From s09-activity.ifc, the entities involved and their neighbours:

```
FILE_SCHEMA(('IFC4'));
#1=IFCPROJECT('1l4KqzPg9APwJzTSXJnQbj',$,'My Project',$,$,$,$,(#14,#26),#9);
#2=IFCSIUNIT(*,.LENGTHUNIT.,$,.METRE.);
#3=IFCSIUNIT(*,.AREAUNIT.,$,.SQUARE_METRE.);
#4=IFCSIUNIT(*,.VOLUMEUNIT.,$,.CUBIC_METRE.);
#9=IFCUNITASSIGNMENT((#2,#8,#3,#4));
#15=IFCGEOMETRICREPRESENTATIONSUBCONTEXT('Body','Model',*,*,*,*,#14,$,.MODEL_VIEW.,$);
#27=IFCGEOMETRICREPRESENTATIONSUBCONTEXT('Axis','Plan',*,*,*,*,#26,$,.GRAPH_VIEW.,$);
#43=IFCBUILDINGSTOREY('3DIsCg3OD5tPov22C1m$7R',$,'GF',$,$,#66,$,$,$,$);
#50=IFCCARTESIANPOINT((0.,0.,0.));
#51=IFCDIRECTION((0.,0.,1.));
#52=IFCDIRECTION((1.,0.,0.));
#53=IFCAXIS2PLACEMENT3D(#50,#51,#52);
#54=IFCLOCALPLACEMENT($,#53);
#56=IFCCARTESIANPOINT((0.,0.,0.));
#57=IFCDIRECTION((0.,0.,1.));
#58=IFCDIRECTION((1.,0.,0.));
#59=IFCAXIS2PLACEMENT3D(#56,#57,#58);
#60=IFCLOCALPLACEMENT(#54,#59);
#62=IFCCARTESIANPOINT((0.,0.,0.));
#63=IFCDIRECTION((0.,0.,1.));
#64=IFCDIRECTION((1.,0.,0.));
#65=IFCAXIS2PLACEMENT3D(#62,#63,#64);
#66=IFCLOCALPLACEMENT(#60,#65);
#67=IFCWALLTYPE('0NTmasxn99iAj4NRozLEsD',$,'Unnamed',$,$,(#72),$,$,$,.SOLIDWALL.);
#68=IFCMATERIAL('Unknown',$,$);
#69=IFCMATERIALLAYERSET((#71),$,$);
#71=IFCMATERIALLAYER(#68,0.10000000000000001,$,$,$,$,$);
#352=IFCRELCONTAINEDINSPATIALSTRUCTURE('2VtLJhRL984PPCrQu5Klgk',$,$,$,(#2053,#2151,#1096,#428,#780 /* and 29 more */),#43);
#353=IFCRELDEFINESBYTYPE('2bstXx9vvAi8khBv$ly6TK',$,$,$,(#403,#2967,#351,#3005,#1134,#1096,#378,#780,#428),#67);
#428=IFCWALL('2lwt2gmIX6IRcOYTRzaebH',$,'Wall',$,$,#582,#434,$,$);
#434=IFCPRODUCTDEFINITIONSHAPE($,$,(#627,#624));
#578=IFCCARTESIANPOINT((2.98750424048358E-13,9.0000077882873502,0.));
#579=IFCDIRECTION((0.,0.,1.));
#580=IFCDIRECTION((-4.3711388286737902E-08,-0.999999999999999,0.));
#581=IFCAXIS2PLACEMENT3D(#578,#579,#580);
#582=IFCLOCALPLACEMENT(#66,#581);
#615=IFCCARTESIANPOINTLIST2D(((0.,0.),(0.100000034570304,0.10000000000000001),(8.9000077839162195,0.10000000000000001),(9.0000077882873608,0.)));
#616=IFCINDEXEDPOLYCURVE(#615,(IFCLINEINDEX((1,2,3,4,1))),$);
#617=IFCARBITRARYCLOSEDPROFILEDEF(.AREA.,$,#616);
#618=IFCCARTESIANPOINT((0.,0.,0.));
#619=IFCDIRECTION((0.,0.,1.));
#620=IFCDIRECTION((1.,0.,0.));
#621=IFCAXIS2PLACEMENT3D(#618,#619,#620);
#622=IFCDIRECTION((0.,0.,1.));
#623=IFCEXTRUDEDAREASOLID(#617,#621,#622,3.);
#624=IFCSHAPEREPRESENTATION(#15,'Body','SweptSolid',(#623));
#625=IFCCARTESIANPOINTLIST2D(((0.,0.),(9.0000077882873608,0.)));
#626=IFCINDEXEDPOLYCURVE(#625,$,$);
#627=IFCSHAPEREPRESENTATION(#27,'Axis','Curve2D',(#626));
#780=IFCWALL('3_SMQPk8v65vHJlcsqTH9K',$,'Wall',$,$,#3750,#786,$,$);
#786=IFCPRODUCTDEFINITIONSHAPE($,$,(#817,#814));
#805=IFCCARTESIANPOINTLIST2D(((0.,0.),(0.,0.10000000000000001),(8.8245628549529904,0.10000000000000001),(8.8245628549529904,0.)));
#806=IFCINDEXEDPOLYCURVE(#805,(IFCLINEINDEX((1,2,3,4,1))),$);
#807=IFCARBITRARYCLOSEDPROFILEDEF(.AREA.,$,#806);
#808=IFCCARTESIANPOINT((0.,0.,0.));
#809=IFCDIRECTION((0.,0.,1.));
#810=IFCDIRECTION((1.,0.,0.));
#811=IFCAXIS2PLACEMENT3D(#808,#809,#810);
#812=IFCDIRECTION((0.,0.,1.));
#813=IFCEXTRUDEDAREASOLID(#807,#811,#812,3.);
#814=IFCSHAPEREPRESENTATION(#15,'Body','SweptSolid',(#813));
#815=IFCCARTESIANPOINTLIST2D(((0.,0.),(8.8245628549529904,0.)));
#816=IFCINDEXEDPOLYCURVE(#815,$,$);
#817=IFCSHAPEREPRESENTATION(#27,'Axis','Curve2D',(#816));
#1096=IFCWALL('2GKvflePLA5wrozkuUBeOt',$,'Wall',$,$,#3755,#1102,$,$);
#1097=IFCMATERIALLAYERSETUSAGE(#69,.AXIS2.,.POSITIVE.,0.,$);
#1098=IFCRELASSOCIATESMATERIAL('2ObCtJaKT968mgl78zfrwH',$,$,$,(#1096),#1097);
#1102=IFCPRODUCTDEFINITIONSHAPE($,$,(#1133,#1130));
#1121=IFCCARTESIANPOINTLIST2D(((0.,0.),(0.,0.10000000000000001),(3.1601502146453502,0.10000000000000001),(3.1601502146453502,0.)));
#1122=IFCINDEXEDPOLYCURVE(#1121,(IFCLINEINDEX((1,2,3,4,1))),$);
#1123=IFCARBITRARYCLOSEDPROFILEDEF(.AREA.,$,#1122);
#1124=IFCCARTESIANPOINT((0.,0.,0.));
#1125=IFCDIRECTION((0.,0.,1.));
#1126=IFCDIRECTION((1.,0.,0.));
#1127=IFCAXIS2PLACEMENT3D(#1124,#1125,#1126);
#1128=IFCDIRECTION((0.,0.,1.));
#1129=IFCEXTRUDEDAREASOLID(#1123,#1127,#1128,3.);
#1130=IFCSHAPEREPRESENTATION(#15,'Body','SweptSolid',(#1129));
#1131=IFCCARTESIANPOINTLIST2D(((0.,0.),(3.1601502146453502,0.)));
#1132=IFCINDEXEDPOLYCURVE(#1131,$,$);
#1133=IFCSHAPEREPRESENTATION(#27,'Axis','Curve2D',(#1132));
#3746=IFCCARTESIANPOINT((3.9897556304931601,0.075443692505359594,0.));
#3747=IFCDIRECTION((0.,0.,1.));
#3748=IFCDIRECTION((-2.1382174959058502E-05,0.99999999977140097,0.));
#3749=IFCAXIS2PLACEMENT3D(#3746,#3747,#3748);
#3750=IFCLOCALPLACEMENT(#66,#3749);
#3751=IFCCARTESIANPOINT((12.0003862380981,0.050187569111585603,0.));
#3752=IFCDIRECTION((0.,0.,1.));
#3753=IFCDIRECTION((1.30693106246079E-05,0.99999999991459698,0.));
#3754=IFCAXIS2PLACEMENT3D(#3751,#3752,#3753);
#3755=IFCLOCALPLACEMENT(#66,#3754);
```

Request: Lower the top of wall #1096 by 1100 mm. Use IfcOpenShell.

```python
import ifcopenshell
import ifcopenshell.geom
import ifcopenshell.util.representation
import ifcopenshell.util.shape
import ifcopenshell.util.unit

model = ifcopenshell.open("s09-activity.ifc")
unit_scale = ifcopenshell.util.unit.calculate_unit_scale(model)
settings = ifcopenshell.geom.settings()


def volume(element):
    """Net volume in cubic metres, openings subtracted."""
    shape = ifcopenshell.geom.create_shape(settings, element)
    return ifcopenshell.util.shape.get_volume(shape.geometry)


wall = model.by_id(1096)
before = volume(wall)

body = ifcopenshell.util.representation.get_representation(wall, "Model", "Body")
solid = body.Items[0]
old_height = solid.Depth
solid.Depth -= 1.1 / unit_scale
after = volume(wall)

print(f"height {old_height:g} -> {solid.Depth:g}, volume {before:.3f} -> {after:.3f} m3")

model.write("s09-activity_edited.ifc")
```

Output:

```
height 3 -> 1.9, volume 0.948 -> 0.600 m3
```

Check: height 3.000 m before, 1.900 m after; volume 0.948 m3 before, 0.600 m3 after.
